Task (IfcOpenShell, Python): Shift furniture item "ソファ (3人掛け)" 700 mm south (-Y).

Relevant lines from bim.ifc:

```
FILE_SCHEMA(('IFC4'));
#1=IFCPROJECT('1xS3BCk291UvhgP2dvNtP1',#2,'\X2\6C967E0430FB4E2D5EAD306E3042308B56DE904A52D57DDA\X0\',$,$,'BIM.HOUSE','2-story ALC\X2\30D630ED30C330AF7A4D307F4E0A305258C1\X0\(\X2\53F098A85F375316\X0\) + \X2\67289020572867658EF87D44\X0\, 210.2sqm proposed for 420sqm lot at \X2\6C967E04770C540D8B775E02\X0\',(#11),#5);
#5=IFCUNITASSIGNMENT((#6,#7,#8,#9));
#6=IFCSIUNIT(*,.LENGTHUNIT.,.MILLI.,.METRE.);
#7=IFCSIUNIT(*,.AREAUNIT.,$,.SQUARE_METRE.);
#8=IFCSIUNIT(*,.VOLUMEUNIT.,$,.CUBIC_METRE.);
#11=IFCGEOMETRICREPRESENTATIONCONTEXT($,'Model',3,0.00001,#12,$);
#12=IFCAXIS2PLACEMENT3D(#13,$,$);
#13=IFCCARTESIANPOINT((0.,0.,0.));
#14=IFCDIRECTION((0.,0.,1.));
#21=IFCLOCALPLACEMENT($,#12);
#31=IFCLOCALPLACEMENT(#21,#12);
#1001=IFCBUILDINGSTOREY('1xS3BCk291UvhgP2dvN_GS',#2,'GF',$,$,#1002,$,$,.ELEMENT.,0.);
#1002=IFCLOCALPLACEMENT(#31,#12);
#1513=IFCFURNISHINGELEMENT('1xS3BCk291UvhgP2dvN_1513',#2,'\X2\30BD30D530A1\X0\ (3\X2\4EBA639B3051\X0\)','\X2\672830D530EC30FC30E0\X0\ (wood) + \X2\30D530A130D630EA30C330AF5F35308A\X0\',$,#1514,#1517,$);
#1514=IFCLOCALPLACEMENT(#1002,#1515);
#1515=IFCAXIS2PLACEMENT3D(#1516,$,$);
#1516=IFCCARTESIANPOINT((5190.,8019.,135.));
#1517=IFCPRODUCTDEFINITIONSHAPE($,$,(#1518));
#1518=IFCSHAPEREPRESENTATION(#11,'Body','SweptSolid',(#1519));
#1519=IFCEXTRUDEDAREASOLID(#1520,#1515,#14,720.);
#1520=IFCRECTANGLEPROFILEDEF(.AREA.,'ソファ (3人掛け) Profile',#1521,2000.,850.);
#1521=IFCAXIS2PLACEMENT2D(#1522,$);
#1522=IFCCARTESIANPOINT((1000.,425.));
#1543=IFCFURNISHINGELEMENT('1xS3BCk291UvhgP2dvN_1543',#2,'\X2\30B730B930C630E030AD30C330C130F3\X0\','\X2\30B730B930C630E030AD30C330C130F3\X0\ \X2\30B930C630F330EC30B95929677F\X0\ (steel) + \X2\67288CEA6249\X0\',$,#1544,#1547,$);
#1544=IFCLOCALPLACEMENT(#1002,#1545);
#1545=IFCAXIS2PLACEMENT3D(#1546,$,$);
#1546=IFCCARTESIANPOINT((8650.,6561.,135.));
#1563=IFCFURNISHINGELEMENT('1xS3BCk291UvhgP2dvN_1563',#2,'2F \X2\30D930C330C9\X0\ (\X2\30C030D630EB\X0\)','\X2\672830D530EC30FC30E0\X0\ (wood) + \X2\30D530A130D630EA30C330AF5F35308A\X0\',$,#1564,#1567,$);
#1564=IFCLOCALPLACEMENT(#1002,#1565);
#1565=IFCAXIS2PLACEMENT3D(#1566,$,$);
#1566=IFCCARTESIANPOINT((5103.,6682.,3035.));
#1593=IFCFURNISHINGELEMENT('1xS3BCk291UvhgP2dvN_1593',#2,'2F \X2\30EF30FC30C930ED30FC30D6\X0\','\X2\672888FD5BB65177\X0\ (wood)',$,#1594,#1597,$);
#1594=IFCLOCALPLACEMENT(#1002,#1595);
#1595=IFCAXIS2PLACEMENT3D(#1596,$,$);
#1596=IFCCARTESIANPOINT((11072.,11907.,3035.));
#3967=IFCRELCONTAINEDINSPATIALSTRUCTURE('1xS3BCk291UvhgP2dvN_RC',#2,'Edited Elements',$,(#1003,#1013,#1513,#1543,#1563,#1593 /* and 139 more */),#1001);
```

```python
import ifcopenshell
import ifcopenshell.api.geometry
import ifcopenshell.util.placement

model = ifcopenshell.open("bim.ifc")

item = model.by_id(1513)
matrix = ifcopenshell.util.placement.get_local_placement(item.ObjectPlacement)
matrix[1, 3] -= 700.0
ifcopenshell.api.geometry.edit_object_placement(model, product=item, matrix=matrix, is_si=False)

print(ifcopenshell.util.placement.get_local_placement(item.ObjectPlacement).round(3) + 0.0)

model.write("bim-out.ifc")
```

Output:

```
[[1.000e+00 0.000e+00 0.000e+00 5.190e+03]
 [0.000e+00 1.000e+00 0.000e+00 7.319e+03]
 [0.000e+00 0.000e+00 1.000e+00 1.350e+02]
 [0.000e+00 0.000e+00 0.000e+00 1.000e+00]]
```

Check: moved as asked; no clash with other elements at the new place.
